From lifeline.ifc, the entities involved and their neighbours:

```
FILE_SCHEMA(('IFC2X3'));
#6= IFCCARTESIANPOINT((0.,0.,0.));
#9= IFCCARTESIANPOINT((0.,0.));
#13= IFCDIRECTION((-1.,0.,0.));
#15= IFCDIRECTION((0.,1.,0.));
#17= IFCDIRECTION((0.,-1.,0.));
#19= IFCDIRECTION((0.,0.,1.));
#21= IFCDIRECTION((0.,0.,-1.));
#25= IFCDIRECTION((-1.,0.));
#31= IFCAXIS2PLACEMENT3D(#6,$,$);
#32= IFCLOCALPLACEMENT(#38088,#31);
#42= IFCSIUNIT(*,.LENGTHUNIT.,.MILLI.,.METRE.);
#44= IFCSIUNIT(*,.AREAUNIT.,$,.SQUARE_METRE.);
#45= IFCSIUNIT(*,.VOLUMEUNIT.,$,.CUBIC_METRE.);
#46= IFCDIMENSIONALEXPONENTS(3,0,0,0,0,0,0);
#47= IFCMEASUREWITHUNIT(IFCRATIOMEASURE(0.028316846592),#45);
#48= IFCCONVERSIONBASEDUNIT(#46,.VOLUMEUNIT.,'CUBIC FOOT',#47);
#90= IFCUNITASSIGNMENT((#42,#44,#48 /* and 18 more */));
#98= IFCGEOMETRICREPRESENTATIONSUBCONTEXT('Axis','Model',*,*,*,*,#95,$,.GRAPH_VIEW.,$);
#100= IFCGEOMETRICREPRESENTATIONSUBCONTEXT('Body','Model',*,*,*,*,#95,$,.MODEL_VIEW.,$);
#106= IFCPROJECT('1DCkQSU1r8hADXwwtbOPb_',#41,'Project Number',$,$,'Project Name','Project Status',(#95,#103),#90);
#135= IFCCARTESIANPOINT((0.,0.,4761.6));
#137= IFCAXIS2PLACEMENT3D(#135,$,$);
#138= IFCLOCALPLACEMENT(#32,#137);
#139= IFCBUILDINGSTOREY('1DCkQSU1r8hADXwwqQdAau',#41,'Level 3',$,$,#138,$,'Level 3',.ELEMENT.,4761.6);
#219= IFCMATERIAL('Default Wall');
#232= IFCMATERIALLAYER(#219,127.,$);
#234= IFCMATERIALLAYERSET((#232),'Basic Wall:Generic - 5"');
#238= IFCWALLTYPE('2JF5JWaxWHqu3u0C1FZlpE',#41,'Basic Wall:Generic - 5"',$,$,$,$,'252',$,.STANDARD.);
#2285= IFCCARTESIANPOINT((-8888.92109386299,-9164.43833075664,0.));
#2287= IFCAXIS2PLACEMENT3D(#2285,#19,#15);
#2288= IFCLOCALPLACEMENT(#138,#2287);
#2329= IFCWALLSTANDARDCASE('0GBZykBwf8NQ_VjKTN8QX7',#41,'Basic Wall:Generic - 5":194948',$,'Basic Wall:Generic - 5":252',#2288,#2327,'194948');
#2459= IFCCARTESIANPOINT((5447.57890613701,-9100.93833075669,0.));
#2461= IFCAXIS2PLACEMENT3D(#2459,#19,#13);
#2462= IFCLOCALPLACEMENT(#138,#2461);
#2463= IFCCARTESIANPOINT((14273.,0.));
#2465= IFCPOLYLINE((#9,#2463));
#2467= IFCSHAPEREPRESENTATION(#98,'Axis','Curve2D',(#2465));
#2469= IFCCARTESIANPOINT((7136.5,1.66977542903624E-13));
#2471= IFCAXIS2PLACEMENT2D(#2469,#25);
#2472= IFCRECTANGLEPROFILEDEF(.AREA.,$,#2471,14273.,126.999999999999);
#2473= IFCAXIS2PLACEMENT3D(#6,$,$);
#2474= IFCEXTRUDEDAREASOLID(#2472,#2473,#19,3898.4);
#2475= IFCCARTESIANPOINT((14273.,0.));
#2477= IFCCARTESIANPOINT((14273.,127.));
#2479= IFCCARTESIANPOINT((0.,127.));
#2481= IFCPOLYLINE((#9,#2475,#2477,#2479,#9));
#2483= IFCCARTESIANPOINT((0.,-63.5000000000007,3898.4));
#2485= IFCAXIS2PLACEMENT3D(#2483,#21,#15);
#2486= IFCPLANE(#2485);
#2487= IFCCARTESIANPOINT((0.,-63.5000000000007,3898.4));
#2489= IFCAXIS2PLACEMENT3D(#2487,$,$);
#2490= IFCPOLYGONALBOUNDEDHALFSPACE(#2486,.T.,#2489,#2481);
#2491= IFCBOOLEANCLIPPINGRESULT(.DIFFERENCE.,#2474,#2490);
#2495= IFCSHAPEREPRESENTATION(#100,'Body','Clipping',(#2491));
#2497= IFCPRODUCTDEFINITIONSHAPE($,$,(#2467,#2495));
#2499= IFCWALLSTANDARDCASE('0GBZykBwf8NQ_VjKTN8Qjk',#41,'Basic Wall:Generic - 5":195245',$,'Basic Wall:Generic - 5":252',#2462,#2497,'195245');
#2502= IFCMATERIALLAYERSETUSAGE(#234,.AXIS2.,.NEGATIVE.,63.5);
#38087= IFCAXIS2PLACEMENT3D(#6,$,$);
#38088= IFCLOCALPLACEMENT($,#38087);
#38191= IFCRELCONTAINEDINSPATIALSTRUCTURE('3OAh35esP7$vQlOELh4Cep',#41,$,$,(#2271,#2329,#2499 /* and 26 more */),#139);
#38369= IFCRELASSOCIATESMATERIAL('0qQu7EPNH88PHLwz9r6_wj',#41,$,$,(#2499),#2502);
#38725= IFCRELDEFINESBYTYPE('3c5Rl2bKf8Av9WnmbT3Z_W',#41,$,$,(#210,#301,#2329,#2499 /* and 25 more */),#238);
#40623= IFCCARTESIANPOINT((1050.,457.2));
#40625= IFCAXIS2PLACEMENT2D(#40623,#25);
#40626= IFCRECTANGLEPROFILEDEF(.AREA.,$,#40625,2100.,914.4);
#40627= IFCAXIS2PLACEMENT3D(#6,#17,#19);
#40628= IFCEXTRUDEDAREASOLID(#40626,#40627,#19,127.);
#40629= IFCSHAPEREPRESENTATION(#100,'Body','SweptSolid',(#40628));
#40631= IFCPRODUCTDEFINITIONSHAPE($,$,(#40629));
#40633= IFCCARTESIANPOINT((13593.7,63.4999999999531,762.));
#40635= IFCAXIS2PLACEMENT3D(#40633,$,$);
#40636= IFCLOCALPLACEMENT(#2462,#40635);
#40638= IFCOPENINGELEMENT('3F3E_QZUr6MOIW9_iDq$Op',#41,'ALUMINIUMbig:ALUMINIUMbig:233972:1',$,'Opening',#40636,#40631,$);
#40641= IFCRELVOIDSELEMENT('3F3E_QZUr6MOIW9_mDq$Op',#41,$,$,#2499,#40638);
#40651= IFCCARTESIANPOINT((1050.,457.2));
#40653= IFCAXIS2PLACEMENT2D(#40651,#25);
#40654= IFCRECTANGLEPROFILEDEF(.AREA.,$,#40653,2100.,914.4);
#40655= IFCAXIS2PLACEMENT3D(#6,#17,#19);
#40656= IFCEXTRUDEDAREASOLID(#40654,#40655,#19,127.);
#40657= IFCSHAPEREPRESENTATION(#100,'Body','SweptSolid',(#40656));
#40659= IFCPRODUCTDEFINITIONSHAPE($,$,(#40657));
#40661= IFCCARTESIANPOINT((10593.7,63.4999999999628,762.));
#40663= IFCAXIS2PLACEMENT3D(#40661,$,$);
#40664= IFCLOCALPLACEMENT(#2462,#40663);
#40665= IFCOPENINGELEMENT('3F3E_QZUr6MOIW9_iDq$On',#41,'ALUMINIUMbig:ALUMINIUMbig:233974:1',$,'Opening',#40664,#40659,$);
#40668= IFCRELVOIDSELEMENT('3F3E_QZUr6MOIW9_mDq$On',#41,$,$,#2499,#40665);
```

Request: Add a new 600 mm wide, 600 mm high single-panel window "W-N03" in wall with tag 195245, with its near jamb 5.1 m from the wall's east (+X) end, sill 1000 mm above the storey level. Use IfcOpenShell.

```python
import numpy as np
import ifcopenshell
import ifcopenshell.api.feature
import ifcopenshell.api.geometry
import ifcopenshell.api.root
import ifcopenshell.api.spatial
import ifcopenshell.api.type
import ifcopenshell.geom
import ifcopenshell.util.element
import ifcopenshell.util.placement
import ifcopenshell.util.representation
import ifcopenshell.util.shape
import ifcopenshell.util.unit

model = ifcopenshell.open("lifeline.ifc")
unit_scale = ifcopenshell.util.unit.calculate_unit_scale(model)
settings = ifcopenshell.geom.settings()


def volume(element):
    """Net volume in cubic metres, openings subtracted."""
    shape = ifcopenshell.geom.create_shape(settings, element)
    return ifcopenshell.util.shape.get_volume(shape.geometry)


wall = model.by_guid("0GBZykBwf8NQ_VjKTN8Qjk")
storey = ifcopenshell.util.element.get_container(wall, ifc_class="IfcBuildingStorey")
context = ifcopenshell.util.representation.get_context(model, "Model", "Body", "MODEL_VIEW")
before = volume(wall)

width, height, from_end, sill = 0.6, 0.6, 5.1, 1  # metres

# The wall runs along its own X axis, and the end named is its -X end.
wall_shape = ifcopenshell.geom.create_shape(settings, wall)
x, y, z = ifcopenshell.util.shape.get_vertices(wall_shape.geometry).T
start = x.min() + from_end
face, thickness = float(y.min()), float(y.max() - y.min())
wall_matrix = ifcopenshell.util.placement.get_local_placement(wall.ObjectPlacement)
level = ifcopenshell.util.placement.get_local_placement(storey.ObjectPlacement)[2, 3]


def in_wall(x, y):
    """Placement at x, y metres in the wall's axes, at sill height."""
    matrix = wall_matrix.copy()
    matrix[:, 3] = wall_matrix @ np.array([x / unit_scale, y / unit_scale, 0.0, 1.0])
    matrix[2, 3] = level + sill / unit_scale
    return matrix


# Opening: a box that overshoots both wall faces by 50 mm.
opening = ifcopenshell.api.root.create_entity(model, ifc_class="IfcOpeningElement")
box = ifcopenshell.api.geometry.add_wall_representation(
    model, context=context, length=width, height=height, thickness=thickness + 0.1
)
ifcopenshell.api.geometry.assign_representation(model, product=opening, representation=box)
ifcopenshell.api.geometry.edit_object_placement(model, product=opening, matrix=in_wall(start, face - 0.05), is_si=False)
ifcopenshell.api.feature.add_feature(model, feature=opening, element=wall)

window = ifcopenshell.api.root.create_entity(model, ifc_class="IfcWindow", name="W-N03")
window.OverallWidth, window.OverallHeight = width / unit_scale, height / unit_scale
body = ifcopenshell.api.geometry.add_window_representation(
    model,
    context=context,
    overall_width=window.OverallWidth,
    overall_height=window.OverallHeight,
    partition_type="SINGLE_PANEL",
)
ifcopenshell.api.geometry.assign_representation(model, product=window, representation=body)
ifcopenshell.api.spatial.assign_container(model, products=[window], relating_structure=storey)
fills = ifcopenshell.api.feature.add_filling(model, opening=opening, element=window)
fills.OwnerHistory = window.OwnerHistory  # required in IFC2X3

# IFC2X3 keeps the operation on the window style.
style = ifcopenshell.api.root.create_entity(model, ifc_class="IfcWindowStyle", name="W-N03")
style.OperationType, style.ConstructionType = "SINGLE_PANEL", "NOTDEFINED"
style.ParameterTakesPrecedence = style.Sizeable = False
ifcopenshell.api.type.assign_type(model, related_objects=[window], relating_type=style)

# Centre the window in the wall's thickness.
ifcopenshell.api.geometry.edit_object_placement(model, product=window, matrix=in_wall(start, face), is_si=False)
window_shape = ifcopenshell.geom.create_shape(settings, window)
depth = ifcopenshell.util.shape.get_vertices(window_shape.geometry)[:, 1]
offset = face + thickness / 2 - (depth.min() + depth.max()) / 2
ifcopenshell.api.geometry.edit_object_placement(model, product=window, matrix=in_wall(start, offset), is_si=False)

after = volume(wall)

print(f"wall volume {before:.3f} -> {after:.3f} m3")

model.write("lifeline_edited.ifc")
```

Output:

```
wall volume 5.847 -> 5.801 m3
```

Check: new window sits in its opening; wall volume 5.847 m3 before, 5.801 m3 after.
